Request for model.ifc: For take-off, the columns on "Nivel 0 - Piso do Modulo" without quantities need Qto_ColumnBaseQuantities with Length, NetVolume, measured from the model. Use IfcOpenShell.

First a look at what the model holds.

```python
import ifcopenshell
import ifcopenshell.util.element
import ifcopenshell.util.unit

model = ifcopenshell.open("model.ifc")
print(model.schema)
for unit_type in ("LENGTHUNIT", "AREAUNIT", "VOLUMEUNIT"):
    print(unit_type, ifcopenshell.util.unit.calculate_unit_scale(model, unit_type))
storey = next(s for s in model.by_type("IfcBuildingStorey") if s.Name == "Nivel 0 - Piso do Modulo")
columns = [e for e in ifcopenshell.util.element.get_decomposition(storey) if e.is_a("IfcColumn")]
for e in sorted(columns, key=lambda e: e.id()):
    print(e.id(), e.is_a(), e.Name, list(ifcopenshell.util.element.get_psets(e, qtos_only=True)), sep=" | ")
```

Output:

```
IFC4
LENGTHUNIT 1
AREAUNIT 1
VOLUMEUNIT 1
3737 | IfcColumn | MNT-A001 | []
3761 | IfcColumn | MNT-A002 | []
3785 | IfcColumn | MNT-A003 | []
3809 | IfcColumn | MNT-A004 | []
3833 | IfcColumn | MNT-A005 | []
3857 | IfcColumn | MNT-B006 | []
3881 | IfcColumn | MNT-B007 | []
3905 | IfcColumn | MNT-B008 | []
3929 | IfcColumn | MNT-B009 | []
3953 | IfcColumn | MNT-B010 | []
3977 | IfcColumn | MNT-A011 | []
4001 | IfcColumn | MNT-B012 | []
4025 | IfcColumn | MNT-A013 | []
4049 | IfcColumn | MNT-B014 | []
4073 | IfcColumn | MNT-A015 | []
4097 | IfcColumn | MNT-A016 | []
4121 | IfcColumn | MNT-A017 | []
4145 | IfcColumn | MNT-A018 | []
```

```python
import ifcopenshell
import ifcopenshell.api.pset
import ifcopenshell.geom
import ifcopenshell.util.element
import ifcopenshell.util.shape
import ifcopenshell.util.unit

model = ifcopenshell.open("model.ifc")
unit_scale = ifcopenshell.util.unit.calculate_unit_scale(model)
volume_scale = ifcopenshell.util.unit.calculate_unit_scale(model, "VOLUMEUNIT")
settings = ifcopenshell.geom.settings()

storey = next(s for s in model.by_type("IfcBuildingStorey") if s.Name == "Nivel 0 - Piso do Modulo")
columns = [e for e in ifcopenshell.util.element.get_decomposition(storey) if e.is_a("IfcColumn")]

for e in sorted(columns, key=lambda e: e.id()):
    if ifcopenshell.util.element.get_psets(e, qtos_only=True, should_inherit=False):
        continue
    # Geometry comes back in metres, in the element's own axes.
    shape = ifcopenshell.geom.create_shape(settings, e)
    values = {
        "Length": ifcopenshell.util.shape.get_z(shape.geometry) / unit_scale,
        "NetVolume": ifcopenshell.util.shape.get_volume(shape.geometry) / volume_scale,
    }
    qto = ifcopenshell.api.pset.add_qto(model, product=e, name="Qto_ColumnBaseQuantities")
    ifcopenshell.api.pset.edit_qto(model, qto=qto, properties=values)
    print(e.id(), {k: round(v, 3) for k, v in values.items()})

model.write("model_updated.ifc")
```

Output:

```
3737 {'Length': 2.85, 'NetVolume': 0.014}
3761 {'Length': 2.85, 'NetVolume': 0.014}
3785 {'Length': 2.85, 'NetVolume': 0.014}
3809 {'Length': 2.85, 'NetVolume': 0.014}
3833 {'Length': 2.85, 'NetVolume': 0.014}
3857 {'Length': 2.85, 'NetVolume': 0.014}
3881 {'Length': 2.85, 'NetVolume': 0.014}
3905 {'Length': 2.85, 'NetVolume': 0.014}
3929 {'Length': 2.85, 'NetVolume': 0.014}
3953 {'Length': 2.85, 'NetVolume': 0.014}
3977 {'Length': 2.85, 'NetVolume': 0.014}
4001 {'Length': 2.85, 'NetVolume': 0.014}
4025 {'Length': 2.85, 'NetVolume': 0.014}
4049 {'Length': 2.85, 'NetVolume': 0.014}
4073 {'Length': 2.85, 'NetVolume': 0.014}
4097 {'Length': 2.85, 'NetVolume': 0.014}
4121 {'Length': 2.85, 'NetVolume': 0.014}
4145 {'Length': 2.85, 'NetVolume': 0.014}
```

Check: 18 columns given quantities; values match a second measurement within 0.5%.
